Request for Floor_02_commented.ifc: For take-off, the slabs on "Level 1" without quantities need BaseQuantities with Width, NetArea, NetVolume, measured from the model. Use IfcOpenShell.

First a look at what the model holds.

```python
import ifcopenshell
import ifcopenshell.util.element
import ifcopenshell.util.unit

model = ifcopenshell.open("Floor_02_commented.ifc")
print(model.schema)
for unit_type in ("LENGTHUNIT", "AREAUNIT", "VOLUMEUNIT"):
    print(unit_type, ifcopenshell.util.unit.calculate_unit_scale(model, unit_type))
storey = next(s for s in model.by_type("IfcBuildingStorey") if s.Name == "Level 1")
slabs = [e for e in ifcopenshell.util.element.get_decomposition(storey) if e.is_a("IfcSlab")]
for e in sorted(slabs, key=lambda e: e.id()):
    print(e.id(), e.is_a(), e.Name, list(ifcopenshell.util.element.get_psets(e, qtos_only=True)), sep=" | ")
```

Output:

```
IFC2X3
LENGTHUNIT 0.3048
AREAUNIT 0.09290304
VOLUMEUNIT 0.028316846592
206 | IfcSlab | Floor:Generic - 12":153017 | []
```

```python
import ifcopenshell
import ifcopenshell.api.pset
import ifcopenshell.geom
import ifcopenshell.util.element
import ifcopenshell.util.shape
import ifcopenshell.util.unit

model = ifcopenshell.open("Floor_02_commented.ifc")
unit_scale = ifcopenshell.util.unit.calculate_unit_scale(model)
area_scale = ifcopenshell.util.unit.calculate_unit_scale(model, "AREAUNIT")
volume_scale = ifcopenshell.util.unit.calculate_unit_scale(model, "VOLUMEUNIT")
settings = ifcopenshell.geom.settings()

storey = next(s for s in model.by_type("IfcBuildingStorey") if s.Name == "Level 1")
slabs = [e for e in ifcopenshell.util.element.get_decomposition(storey) if e.is_a("IfcSlab")]

for e in sorted(slabs, key=lambda e: e.id()):
    if ifcopenshell.util.element.get_psets(e, qtos_only=True, should_inherit=False):
        continue
    # Geometry comes back in metres, in the element's own axes.
    shape = ifcopenshell.geom.create_shape(settings, e)
    values = {
        "Width": ifcopenshell.util.shape.get_z(shape.geometry) / unit_scale,
        "NetArea": ifcopenshell.util.shape.get_footprint_area(shape.geometry) / area_scale,
        "NetVolume": ifcopenshell.util.shape.get_volume(shape.geometry) / volume_scale,
    }
    qto = ifcopenshell.api.pset.add_qto(model, product=e, name="BaseQuantities")
    ifcopenshell.api.pset.edit_qto(model, qto=qto, properties=values)
    print(e.id(), {k: round(v, 3) for k, v in values.items()})

model.write("Floor_02_commented_updated.ifc")
```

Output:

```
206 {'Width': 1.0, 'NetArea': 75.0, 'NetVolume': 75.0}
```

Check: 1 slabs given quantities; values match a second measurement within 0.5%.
